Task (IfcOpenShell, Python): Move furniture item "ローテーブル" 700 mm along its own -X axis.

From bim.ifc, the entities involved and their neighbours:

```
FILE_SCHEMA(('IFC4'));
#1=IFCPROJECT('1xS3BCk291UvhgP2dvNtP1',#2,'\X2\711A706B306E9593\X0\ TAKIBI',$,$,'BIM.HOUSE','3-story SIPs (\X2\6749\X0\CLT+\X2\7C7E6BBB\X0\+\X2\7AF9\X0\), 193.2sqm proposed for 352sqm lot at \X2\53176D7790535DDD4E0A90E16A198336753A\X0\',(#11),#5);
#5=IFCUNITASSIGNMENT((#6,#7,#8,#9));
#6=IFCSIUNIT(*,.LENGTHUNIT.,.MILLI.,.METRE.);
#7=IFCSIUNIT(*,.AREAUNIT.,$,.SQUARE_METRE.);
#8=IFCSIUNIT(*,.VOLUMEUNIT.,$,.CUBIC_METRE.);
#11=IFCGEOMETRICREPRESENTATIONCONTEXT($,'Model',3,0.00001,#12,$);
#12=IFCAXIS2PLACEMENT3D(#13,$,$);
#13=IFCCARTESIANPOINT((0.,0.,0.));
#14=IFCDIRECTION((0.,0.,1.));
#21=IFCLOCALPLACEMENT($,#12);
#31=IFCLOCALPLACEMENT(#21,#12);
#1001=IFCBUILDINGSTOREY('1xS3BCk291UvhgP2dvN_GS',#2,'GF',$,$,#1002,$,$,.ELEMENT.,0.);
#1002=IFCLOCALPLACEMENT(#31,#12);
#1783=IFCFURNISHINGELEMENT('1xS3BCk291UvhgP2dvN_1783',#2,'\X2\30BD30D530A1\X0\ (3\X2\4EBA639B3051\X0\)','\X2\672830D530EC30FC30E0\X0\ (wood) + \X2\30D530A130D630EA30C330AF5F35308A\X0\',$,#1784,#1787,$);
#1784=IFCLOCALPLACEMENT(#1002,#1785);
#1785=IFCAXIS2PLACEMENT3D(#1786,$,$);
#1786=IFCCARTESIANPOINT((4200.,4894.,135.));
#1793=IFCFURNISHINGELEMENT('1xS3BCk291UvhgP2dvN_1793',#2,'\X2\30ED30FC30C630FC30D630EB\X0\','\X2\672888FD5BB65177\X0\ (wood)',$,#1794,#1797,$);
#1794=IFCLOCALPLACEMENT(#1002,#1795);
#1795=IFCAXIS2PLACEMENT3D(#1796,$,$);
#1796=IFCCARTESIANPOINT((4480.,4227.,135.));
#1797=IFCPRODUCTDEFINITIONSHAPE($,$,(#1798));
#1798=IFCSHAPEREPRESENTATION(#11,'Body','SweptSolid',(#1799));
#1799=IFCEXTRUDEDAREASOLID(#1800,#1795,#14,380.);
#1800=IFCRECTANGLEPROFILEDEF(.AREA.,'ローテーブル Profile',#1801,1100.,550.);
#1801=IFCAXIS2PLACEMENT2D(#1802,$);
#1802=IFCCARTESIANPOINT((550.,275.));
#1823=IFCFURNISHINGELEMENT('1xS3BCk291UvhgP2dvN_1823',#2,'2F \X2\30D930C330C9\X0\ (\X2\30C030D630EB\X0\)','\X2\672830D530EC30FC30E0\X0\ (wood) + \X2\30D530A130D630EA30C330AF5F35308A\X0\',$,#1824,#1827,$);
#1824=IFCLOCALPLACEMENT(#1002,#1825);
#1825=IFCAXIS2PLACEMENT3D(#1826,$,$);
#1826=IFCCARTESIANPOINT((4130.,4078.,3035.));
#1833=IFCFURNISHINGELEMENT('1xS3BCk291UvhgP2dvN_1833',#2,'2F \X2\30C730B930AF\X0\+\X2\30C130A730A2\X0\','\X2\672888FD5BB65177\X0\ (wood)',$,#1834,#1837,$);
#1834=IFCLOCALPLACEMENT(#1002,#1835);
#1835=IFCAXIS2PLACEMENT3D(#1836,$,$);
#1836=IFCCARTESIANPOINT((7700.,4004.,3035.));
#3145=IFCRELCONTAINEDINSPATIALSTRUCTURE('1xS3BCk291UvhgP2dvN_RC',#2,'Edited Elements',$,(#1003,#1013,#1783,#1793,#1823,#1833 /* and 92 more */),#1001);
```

```python
import ifcopenshell
import ifcopenshell.api.geometry
import ifcopenshell.util.placement

model = ifcopenshell.open("bim.ifc")

item = model.by_guid("1xS3BCk291UvhgP2dvN_1793")
matrix = ifcopenshell.util.placement.get_local_placement(item.ObjectPlacement)
matrix[:3, 3] -= matrix[:3, 0] * 700.0
ifcopenshell.api.geometry.edit_object_placement(model, product=item, matrix=matrix, is_si=False)

print(ifcopenshell.util.placement.get_local_placement(item.ObjectPlacement).round(3) + 0.0)

model.write("bim_edited.ifc")
```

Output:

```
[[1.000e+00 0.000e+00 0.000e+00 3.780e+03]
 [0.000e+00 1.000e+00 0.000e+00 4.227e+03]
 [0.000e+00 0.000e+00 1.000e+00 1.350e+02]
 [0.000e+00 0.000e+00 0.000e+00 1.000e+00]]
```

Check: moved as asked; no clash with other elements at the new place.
